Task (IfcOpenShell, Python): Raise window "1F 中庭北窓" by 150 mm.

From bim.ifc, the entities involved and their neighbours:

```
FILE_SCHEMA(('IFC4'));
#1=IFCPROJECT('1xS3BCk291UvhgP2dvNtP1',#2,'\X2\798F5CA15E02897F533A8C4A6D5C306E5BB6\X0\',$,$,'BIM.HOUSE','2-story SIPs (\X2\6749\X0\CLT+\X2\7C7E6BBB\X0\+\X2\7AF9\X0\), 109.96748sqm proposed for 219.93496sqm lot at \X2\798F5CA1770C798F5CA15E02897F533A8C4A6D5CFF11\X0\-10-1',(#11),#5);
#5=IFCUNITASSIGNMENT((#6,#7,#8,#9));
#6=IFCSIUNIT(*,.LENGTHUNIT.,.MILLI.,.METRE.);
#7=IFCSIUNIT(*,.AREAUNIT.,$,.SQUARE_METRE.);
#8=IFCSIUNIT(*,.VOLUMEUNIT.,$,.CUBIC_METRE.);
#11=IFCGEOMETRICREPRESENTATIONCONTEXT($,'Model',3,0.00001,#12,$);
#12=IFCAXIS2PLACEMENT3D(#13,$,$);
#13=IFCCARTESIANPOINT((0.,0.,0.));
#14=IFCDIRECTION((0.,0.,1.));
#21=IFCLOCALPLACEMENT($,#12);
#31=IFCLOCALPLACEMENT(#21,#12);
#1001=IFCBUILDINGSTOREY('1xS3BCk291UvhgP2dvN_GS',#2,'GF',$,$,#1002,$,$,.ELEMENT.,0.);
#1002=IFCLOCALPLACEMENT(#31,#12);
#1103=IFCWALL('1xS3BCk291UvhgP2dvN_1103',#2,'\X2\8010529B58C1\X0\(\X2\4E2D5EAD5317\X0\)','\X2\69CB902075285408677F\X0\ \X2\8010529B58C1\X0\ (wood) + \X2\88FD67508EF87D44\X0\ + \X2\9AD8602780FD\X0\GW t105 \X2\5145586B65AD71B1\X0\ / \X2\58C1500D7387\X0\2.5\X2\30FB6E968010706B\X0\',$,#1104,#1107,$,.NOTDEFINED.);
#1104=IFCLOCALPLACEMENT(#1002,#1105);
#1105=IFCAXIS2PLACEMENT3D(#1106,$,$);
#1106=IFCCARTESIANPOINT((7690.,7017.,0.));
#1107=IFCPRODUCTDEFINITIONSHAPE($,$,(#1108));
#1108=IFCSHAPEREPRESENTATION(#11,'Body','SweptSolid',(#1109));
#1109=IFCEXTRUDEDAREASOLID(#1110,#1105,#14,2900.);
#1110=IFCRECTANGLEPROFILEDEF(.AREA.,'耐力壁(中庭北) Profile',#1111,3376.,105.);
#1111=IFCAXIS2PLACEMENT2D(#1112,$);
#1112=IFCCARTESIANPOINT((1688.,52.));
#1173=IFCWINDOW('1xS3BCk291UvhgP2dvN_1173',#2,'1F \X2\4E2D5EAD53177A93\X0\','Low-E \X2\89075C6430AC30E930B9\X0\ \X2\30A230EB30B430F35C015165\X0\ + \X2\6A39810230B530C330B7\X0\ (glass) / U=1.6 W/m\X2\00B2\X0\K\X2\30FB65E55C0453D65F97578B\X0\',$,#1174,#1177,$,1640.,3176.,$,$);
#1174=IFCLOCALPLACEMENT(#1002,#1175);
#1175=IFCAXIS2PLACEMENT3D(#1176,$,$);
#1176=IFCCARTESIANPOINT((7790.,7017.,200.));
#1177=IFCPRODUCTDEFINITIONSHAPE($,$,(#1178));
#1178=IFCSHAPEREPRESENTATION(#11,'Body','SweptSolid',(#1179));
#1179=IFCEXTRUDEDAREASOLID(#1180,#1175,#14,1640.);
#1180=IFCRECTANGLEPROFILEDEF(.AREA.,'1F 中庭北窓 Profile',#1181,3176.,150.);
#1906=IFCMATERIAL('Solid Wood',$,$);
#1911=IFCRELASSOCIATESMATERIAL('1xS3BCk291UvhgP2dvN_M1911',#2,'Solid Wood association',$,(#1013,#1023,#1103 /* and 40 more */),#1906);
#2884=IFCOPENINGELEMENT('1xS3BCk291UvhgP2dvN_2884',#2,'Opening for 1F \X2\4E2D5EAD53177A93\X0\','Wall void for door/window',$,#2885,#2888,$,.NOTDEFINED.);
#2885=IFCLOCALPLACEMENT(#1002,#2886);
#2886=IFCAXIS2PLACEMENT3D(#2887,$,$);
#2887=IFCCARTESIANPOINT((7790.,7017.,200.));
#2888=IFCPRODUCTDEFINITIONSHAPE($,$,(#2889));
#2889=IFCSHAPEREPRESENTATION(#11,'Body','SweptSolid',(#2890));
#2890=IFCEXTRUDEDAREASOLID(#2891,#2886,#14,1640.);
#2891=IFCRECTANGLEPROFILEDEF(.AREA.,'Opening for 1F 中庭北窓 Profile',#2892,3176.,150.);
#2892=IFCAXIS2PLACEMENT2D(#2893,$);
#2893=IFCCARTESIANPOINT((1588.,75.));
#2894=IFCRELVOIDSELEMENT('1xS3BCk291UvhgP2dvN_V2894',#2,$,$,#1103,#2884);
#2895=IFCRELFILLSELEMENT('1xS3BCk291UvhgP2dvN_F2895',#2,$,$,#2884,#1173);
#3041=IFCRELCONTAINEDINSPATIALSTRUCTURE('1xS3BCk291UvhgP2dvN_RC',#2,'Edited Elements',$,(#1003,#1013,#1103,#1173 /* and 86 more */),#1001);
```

```python
import numpy as np
import ifcopenshell
import ifcopenshell.api.geometry
import ifcopenshell.util.placement
import ifcopenshell.util.unit

model = ifcopenshell.open("bim.ifc")
unit_scale = ifcopenshell.util.unit.calculate_unit_scale(model)

window = model.by_guid("1xS3BCk291UvhgP2dvN_1173")
opening = window.FillsVoids[0].RelatingOpeningElement
dz = 0.15 / unit_scale

shift = np.array([0.0, 0.0, dz])
# The window is not placed relative to its opening, so move both.
for product in (opening, window):
    matrix = ifcopenshell.util.placement.get_local_placement(product.ObjectPlacement)
    matrix[:3, 3] += shift
    ifcopenshell.api.geometry.edit_object_placement(model, product=product, matrix=matrix, is_si=False)

print(f"moved by {dz * unit_scale:+.3f} m")

model.write("bim_edited.ifc")
```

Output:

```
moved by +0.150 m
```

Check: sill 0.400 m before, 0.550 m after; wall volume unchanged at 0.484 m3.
